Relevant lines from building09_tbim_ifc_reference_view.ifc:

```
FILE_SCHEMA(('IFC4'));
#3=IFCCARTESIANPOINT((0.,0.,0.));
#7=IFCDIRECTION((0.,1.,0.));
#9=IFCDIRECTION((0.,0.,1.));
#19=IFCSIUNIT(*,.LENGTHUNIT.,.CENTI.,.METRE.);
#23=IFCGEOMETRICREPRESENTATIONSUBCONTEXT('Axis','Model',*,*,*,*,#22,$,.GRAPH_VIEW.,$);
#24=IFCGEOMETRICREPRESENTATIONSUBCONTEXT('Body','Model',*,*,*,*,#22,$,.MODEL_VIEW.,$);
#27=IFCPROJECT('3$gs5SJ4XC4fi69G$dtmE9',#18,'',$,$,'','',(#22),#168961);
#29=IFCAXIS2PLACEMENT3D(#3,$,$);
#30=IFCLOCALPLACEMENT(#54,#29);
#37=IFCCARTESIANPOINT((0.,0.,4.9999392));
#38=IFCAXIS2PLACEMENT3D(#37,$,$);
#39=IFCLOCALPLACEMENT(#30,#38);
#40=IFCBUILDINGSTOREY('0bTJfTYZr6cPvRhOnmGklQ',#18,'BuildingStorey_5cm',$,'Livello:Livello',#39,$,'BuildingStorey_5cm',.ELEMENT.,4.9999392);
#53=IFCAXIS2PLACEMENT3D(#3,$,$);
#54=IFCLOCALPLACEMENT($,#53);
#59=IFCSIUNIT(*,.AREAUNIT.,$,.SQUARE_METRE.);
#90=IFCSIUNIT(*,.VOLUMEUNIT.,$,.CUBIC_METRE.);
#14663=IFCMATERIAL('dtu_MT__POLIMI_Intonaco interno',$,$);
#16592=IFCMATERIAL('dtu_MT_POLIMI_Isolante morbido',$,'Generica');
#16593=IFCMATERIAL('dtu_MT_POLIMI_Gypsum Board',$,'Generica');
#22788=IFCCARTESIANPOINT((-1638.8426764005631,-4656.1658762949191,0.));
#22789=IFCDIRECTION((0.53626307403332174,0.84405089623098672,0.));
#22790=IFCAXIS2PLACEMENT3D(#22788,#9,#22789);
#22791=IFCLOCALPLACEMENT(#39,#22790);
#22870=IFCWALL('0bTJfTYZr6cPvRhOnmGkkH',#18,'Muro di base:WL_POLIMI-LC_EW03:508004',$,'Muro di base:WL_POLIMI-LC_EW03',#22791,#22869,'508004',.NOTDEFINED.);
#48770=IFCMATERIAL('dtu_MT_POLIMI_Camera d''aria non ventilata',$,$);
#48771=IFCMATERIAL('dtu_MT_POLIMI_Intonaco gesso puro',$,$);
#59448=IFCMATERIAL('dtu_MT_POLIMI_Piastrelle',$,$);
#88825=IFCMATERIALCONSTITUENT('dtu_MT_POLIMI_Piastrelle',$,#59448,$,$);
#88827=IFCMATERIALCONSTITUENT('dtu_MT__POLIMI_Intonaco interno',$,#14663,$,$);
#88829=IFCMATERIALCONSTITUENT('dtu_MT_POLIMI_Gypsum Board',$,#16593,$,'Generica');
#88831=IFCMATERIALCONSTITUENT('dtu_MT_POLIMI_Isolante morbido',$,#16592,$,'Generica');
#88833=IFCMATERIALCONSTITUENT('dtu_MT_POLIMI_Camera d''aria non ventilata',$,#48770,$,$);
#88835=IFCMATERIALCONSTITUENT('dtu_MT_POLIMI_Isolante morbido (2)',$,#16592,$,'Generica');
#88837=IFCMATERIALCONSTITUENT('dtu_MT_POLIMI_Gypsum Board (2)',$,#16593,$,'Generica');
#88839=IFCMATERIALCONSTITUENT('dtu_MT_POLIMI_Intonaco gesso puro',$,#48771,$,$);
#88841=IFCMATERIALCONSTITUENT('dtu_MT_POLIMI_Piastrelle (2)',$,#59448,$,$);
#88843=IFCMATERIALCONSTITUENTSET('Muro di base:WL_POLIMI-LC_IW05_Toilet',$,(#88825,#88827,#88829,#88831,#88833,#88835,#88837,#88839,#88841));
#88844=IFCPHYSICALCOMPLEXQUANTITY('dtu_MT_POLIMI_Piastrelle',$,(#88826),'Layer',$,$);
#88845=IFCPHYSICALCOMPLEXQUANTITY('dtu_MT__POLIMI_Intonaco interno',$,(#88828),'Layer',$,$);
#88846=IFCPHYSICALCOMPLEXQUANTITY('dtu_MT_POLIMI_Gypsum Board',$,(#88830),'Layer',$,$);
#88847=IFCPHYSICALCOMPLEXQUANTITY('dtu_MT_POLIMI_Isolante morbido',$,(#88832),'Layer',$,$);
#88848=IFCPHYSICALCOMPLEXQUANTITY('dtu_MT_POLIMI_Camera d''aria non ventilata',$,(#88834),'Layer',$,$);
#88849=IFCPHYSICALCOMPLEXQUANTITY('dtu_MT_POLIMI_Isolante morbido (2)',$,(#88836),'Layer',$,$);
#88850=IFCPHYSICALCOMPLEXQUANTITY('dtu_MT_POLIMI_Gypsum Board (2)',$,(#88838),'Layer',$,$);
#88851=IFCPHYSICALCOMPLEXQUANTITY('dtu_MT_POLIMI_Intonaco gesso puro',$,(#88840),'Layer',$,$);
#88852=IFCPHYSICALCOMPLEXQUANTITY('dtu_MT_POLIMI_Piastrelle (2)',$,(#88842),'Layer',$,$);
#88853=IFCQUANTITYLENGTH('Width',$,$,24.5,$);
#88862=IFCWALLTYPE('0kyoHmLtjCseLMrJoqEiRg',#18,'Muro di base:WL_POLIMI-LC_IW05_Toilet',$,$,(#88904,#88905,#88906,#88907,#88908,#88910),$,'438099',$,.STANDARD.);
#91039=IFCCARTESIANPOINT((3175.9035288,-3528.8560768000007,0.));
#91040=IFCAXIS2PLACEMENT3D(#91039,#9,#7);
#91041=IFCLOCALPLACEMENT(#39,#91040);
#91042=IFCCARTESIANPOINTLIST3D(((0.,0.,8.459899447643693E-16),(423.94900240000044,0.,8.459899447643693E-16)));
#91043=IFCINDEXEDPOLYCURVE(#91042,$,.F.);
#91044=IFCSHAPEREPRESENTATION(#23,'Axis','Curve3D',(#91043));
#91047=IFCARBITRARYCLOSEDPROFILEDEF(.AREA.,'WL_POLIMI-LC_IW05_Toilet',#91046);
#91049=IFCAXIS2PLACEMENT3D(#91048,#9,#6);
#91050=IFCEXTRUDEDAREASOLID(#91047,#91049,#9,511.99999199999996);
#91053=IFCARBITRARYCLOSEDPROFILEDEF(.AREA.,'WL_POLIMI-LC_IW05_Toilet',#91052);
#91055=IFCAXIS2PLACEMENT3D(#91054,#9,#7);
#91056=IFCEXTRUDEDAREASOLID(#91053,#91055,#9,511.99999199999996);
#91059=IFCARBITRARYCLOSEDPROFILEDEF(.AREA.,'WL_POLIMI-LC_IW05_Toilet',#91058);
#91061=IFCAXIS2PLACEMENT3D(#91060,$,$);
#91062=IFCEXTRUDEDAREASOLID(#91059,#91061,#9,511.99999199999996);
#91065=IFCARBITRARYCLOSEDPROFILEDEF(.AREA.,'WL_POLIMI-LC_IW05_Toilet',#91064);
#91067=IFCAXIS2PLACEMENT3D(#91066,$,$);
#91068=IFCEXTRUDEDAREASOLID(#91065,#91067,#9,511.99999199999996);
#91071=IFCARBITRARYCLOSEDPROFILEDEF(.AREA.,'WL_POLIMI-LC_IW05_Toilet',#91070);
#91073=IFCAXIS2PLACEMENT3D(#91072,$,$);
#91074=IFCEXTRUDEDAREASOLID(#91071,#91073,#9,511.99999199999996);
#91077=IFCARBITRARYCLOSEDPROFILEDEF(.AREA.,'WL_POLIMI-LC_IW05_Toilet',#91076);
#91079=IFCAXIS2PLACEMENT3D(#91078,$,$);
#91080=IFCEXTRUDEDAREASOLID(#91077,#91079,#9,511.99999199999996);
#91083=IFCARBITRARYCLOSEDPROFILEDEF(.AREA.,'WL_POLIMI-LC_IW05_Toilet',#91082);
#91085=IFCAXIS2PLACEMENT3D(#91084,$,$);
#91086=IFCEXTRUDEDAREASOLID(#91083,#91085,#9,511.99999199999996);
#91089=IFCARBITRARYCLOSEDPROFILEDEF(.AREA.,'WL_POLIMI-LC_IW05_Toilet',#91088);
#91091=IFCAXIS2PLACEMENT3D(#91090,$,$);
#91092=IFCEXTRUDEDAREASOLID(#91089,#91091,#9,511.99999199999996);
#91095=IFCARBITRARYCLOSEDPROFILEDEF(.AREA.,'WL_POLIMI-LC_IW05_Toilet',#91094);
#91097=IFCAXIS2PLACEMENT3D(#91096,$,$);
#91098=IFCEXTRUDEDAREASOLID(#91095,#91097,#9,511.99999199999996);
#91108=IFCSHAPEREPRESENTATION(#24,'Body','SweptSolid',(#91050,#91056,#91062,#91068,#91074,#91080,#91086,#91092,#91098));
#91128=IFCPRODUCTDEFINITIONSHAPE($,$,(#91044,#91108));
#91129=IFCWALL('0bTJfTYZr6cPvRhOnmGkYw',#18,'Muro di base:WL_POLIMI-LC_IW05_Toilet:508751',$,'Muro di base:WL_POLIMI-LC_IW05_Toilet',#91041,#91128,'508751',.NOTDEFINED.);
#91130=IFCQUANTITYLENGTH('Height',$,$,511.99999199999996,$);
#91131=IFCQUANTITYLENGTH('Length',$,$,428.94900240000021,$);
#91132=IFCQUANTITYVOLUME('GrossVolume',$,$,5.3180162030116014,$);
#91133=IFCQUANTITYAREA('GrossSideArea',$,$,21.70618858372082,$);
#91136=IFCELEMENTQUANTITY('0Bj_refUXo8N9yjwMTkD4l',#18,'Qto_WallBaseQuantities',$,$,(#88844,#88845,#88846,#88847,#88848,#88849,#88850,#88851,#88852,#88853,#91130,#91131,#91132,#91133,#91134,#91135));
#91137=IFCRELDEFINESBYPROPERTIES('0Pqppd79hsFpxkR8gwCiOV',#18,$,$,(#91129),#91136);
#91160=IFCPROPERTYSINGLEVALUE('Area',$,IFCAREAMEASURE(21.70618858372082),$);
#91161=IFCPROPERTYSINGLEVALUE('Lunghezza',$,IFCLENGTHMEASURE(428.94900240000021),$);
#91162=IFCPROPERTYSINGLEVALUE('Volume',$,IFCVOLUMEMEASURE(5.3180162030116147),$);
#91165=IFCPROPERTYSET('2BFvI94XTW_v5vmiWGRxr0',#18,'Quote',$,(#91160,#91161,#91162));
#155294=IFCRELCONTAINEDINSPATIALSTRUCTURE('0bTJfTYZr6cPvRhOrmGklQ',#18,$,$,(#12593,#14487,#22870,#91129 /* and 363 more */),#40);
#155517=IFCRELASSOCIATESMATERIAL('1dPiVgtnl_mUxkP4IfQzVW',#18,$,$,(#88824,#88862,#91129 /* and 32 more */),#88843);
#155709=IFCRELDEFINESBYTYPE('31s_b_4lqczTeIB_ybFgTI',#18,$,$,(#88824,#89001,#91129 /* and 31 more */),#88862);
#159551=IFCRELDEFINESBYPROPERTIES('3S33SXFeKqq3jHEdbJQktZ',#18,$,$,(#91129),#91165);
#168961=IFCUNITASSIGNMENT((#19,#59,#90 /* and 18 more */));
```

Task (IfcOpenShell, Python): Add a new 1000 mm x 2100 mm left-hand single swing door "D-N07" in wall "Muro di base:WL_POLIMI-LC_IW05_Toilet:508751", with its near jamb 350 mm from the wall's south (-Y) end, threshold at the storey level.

```python
import numpy as np
import ifcopenshell
import ifcopenshell.api.feature
import ifcopenshell.api.geometry
import ifcopenshell.api.pset
import ifcopenshell.api.root
import ifcopenshell.api.spatial
import ifcopenshell.geom
import ifcopenshell.util.element
import ifcopenshell.util.placement
import ifcopenshell.util.representation
import ifcopenshell.util.shape
import ifcopenshell.util.unit

model = ifcopenshell.open("building09_tbim_ifc_reference_view.ifc")
unit_scale = ifcopenshell.util.unit.calculate_unit_scale(model)
area_scale = ifcopenshell.util.unit.calculate_unit_scale(model, "AREAUNIT")
volume_scale = ifcopenshell.util.unit.calculate_unit_scale(model, "VOLUMEUNIT")
settings = ifcopenshell.geom.settings()


def volume(element):
    """Net volume in cubic metres, openings subtracted."""
    shape = ifcopenshell.geom.create_shape(settings, element)
    return ifcopenshell.util.shape.get_volume(shape.geometry)


wall = model.by_guid("0bTJfTYZr6cPvRhOnmGkYw")
storey = ifcopenshell.util.element.get_container(wall, ifc_class="IfcBuildingStorey")
context = ifcopenshell.util.representation.get_context(model, "Model", "Body", "MODEL_VIEW")
before = volume(wall)

width, height, from_end, sill = 1, 2.1, 0.35, 0.0  # metres

# The wall runs along its own X axis, and the end named is its -X end.
wall_shape = ifcopenshell.geom.create_shape(settings, wall)
x, y, z = ifcopenshell.util.shape.get_vertices(wall_shape.geometry).T
start = x.min() + from_end
face, thickness = float(y.min()), float(y.max() - y.min())
wall_matrix = ifcopenshell.util.placement.get_local_placement(wall.ObjectPlacement)
level = ifcopenshell.util.placement.get_local_placement(storey.ObjectPlacement)[2, 3]


def in_wall(x, y):
    """Placement at x, y metres in the wall's axes, at sill height."""
    matrix = wall_matrix.copy()
    matrix[:, 3] = wall_matrix @ np.array([x / unit_scale, y / unit_scale, 0.0, 1.0])
    matrix[2, 3] = level + sill / unit_scale
    return matrix


# Opening: a box that overshoots both wall faces by 50 mm.
opening = ifcopenshell.api.root.create_entity(model, ifc_class="IfcOpeningElement", predefined_type="OPENING")
box = ifcopenshell.api.geometry.add_wall_representation(
    model, context=context, length=width, height=height, thickness=thickness + 0.1
)
ifcopenshell.api.geometry.assign_representation(model, product=opening, representation=box)
ifcopenshell.api.geometry.edit_object_placement(model, product=opening, matrix=in_wall(start, face - 0.05), is_si=False)
ifcopenshell.api.feature.add_feature(model, feature=opening, element=wall)

door = ifcopenshell.api.root.create_entity(model, ifc_class="IfcDoor", name="D-N07", predefined_type="DOOR")
door.OverallWidth, door.OverallHeight = width / unit_scale, height / unit_scale
door.OperationType = "SINGLE_SWING_LEFT"
body = ifcopenshell.api.geometry.add_door_representation(
    model,
    context=context,
    overall_width=door.OverallWidth,
    overall_height=door.OverallHeight,
    operation_type="SINGLE_SWING_LEFT",
    lining_properties={"LiningDepth": thickness / unit_scale, "ThresholdDepth": thickness / unit_scale},
)
ifcopenshell.api.geometry.assign_representation(model, product=door, representation=body)
ifcopenshell.api.spatial.assign_container(model, products=[door], relating_structure=storey)
ifcopenshell.api.feature.add_filling(model, opening=opening, element=door)

# The lining spans the wall, so the door starts at the wall face.
ifcopenshell.api.geometry.edit_object_placement(model, product=door, matrix=in_wall(start, face), is_si=False)

after = volume(wall)

# Update the wall's stored quantities.
qto = model.by_id(ifcopenshell.util.element.get_pset(wall, "Qto_WallBaseQuantities", should_inherit=False)["id"])
ifcopenshell.api.pset.edit_qto(model, qto=qto, properties={
    "NetSideArea": after / thickness / area_scale,
    "NetVolume": after / volume_scale,
})
pset = model.by_id(ifcopenshell.util.element.get_pset(wall, "Quote", should_inherit=False)["id"])
ifcopenshell.api.pset.edit_pset(model, pset=pset, properties={
    "Area": model.create_entity("IfcAreaMeasure", after / thickness / area_scale),
    "Volume": model.create_entity("IfcVolumeMeasure", after / volume_scale),
})

print(f"wall volume {before:.3f} -> {after:.3f} m3")

model.write("building09_tbim_ifc_reference_view_edited.ifc")
```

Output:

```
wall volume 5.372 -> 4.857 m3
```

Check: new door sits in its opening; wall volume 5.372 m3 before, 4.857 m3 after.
